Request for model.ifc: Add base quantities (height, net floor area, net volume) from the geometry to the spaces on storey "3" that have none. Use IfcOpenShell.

First a look at what the model holds.

```python
import ifcopenshell
import ifcopenshell.util.element
import ifcopenshell.util.unit

model = ifcopenshell.open("model.ifc")
print(model.schema)
for unit_type in ("LENGTHUNIT", "AREAUNIT", "VOLUMEUNIT"):
    print(unit_type, ifcopenshell.util.unit.calculate_unit_scale(model, unit_type))
storey = next(s for s in model.by_type("IfcBuildingStorey") if s.Name == "3")
spaces = [e for e in ifcopenshell.util.element.get_decomposition(storey) if e.is_a("IfcSpace")]
for e in sorted(spaces, key=lambda e: e.id()):
    print(e.id(), e.is_a(), e.Name, list(ifcopenshell.util.element.get_psets(e, qtos_only=True)), sep=" | ")
```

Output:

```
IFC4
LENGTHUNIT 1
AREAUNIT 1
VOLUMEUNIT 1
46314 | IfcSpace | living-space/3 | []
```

```python
import ifcopenshell
import ifcopenshell.api.pset
import ifcopenshell.geom
import ifcopenshell.util.element
import ifcopenshell.util.shape
import ifcopenshell.util.unit

model = ifcopenshell.open("model.ifc")
unit_scale = ifcopenshell.util.unit.calculate_unit_scale(model)
area_scale = ifcopenshell.util.unit.calculate_unit_scale(model, "AREAUNIT")
volume_scale = ifcopenshell.util.unit.calculate_unit_scale(model, "VOLUMEUNIT")
settings = ifcopenshell.geom.settings()

storey = next(s for s in model.by_type("IfcBuildingStorey") if s.Name == "3")
spaces = [e for e in ifcopenshell.util.element.get_decomposition(storey) if e.is_a("IfcSpace")]

for e in sorted(spaces, key=lambda e: e.id()):
    if ifcopenshell.util.element.get_psets(e, qtos_only=True, should_inherit=False):
        continue
    # Geometry comes back in metres, in the element's own axes.
    shape = ifcopenshell.geom.create_shape(settings, e)
    values = {
        "Height": ifcopenshell.util.shape.get_z(shape.geometry) / unit_scale,
        "NetFloorArea": ifcopenshell.util.shape.get_footprint_area(shape.geometry) / area_scale,
        "NetVolume": ifcopenshell.util.shape.get_volume(shape.geometry) / volume_scale,
    }
    qto = ifcopenshell.api.pset.add_qto(model, product=e, name="Qto_SpaceBaseQuantities")
    ifcopenshell.api.pset.edit_qto(model, qto=qto, properties=values)
    print(e.id(), {k: round(v, 3) for k, v in values.items()})

model.write("model_v2.ifc")
```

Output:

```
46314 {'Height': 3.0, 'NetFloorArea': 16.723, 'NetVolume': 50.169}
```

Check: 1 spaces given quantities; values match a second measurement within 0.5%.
